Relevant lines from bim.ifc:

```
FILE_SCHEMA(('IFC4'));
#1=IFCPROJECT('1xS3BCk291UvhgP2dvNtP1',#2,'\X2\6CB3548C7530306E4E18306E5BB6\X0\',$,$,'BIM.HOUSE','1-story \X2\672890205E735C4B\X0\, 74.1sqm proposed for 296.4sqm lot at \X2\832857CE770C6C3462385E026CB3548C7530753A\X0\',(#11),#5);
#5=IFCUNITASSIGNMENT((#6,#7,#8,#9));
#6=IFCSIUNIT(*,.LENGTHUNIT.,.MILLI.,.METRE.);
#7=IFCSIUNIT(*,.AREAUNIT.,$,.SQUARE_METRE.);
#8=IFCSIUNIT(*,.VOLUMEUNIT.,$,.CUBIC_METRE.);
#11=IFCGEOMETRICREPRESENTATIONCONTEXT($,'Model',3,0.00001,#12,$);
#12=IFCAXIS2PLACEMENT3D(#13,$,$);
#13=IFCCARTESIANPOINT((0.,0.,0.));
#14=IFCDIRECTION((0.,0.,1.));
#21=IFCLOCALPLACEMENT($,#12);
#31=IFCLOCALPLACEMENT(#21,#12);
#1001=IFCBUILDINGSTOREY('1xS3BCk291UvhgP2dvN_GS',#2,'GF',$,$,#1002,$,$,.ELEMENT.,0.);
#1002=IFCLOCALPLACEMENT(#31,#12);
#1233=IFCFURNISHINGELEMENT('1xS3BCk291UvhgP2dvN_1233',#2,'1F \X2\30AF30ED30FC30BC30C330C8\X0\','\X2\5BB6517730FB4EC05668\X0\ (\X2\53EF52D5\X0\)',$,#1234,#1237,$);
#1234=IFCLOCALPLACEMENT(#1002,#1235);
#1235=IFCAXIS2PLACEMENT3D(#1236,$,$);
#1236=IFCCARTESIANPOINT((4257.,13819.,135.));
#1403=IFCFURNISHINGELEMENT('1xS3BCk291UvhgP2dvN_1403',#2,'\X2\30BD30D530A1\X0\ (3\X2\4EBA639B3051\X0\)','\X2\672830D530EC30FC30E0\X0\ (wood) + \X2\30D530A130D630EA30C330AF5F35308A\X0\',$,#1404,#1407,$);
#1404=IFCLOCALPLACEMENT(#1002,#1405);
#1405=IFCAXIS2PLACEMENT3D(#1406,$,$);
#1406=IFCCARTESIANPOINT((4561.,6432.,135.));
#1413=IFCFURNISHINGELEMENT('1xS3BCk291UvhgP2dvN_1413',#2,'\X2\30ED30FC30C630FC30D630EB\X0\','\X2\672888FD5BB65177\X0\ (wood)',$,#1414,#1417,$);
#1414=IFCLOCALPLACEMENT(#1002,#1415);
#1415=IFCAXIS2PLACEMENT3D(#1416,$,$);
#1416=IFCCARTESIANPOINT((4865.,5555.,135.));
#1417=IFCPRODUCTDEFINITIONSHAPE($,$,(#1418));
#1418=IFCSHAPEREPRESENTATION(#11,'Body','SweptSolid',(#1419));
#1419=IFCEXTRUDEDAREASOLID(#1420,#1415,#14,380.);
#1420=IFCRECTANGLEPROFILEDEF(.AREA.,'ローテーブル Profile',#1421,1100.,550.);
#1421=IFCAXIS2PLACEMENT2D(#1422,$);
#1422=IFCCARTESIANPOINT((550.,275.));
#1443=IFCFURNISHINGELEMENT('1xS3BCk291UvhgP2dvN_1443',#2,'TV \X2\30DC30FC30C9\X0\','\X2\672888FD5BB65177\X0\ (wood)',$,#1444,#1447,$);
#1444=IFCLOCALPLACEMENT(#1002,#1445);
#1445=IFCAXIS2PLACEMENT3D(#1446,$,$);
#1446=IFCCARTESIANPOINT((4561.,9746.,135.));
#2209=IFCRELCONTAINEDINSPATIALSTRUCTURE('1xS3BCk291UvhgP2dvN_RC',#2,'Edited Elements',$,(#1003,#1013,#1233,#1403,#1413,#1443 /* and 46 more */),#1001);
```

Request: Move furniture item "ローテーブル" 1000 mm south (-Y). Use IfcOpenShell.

```python
import ifcopenshell
import ifcopenshell.api.geometry
import ifcopenshell.util.placement

model = ifcopenshell.open("bim.ifc")

item = model.by_guid("1xS3BCk291UvhgP2dvN_1413")
matrix = ifcopenshell.util.placement.get_local_placement(item.ObjectPlacement)
matrix[1, 3] -= 1000.0
ifcopenshell.api.geometry.edit_object_placement(model, product=item, matrix=matrix, is_si=False)

print(ifcopenshell.util.placement.get_local_placement(item.ObjectPlacement).round(3) + 0.0)

model.write("bim_edited.ifc")
```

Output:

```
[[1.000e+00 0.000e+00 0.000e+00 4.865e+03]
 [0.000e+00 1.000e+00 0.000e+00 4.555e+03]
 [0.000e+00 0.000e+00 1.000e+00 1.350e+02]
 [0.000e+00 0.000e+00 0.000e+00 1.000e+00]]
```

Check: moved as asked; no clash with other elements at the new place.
